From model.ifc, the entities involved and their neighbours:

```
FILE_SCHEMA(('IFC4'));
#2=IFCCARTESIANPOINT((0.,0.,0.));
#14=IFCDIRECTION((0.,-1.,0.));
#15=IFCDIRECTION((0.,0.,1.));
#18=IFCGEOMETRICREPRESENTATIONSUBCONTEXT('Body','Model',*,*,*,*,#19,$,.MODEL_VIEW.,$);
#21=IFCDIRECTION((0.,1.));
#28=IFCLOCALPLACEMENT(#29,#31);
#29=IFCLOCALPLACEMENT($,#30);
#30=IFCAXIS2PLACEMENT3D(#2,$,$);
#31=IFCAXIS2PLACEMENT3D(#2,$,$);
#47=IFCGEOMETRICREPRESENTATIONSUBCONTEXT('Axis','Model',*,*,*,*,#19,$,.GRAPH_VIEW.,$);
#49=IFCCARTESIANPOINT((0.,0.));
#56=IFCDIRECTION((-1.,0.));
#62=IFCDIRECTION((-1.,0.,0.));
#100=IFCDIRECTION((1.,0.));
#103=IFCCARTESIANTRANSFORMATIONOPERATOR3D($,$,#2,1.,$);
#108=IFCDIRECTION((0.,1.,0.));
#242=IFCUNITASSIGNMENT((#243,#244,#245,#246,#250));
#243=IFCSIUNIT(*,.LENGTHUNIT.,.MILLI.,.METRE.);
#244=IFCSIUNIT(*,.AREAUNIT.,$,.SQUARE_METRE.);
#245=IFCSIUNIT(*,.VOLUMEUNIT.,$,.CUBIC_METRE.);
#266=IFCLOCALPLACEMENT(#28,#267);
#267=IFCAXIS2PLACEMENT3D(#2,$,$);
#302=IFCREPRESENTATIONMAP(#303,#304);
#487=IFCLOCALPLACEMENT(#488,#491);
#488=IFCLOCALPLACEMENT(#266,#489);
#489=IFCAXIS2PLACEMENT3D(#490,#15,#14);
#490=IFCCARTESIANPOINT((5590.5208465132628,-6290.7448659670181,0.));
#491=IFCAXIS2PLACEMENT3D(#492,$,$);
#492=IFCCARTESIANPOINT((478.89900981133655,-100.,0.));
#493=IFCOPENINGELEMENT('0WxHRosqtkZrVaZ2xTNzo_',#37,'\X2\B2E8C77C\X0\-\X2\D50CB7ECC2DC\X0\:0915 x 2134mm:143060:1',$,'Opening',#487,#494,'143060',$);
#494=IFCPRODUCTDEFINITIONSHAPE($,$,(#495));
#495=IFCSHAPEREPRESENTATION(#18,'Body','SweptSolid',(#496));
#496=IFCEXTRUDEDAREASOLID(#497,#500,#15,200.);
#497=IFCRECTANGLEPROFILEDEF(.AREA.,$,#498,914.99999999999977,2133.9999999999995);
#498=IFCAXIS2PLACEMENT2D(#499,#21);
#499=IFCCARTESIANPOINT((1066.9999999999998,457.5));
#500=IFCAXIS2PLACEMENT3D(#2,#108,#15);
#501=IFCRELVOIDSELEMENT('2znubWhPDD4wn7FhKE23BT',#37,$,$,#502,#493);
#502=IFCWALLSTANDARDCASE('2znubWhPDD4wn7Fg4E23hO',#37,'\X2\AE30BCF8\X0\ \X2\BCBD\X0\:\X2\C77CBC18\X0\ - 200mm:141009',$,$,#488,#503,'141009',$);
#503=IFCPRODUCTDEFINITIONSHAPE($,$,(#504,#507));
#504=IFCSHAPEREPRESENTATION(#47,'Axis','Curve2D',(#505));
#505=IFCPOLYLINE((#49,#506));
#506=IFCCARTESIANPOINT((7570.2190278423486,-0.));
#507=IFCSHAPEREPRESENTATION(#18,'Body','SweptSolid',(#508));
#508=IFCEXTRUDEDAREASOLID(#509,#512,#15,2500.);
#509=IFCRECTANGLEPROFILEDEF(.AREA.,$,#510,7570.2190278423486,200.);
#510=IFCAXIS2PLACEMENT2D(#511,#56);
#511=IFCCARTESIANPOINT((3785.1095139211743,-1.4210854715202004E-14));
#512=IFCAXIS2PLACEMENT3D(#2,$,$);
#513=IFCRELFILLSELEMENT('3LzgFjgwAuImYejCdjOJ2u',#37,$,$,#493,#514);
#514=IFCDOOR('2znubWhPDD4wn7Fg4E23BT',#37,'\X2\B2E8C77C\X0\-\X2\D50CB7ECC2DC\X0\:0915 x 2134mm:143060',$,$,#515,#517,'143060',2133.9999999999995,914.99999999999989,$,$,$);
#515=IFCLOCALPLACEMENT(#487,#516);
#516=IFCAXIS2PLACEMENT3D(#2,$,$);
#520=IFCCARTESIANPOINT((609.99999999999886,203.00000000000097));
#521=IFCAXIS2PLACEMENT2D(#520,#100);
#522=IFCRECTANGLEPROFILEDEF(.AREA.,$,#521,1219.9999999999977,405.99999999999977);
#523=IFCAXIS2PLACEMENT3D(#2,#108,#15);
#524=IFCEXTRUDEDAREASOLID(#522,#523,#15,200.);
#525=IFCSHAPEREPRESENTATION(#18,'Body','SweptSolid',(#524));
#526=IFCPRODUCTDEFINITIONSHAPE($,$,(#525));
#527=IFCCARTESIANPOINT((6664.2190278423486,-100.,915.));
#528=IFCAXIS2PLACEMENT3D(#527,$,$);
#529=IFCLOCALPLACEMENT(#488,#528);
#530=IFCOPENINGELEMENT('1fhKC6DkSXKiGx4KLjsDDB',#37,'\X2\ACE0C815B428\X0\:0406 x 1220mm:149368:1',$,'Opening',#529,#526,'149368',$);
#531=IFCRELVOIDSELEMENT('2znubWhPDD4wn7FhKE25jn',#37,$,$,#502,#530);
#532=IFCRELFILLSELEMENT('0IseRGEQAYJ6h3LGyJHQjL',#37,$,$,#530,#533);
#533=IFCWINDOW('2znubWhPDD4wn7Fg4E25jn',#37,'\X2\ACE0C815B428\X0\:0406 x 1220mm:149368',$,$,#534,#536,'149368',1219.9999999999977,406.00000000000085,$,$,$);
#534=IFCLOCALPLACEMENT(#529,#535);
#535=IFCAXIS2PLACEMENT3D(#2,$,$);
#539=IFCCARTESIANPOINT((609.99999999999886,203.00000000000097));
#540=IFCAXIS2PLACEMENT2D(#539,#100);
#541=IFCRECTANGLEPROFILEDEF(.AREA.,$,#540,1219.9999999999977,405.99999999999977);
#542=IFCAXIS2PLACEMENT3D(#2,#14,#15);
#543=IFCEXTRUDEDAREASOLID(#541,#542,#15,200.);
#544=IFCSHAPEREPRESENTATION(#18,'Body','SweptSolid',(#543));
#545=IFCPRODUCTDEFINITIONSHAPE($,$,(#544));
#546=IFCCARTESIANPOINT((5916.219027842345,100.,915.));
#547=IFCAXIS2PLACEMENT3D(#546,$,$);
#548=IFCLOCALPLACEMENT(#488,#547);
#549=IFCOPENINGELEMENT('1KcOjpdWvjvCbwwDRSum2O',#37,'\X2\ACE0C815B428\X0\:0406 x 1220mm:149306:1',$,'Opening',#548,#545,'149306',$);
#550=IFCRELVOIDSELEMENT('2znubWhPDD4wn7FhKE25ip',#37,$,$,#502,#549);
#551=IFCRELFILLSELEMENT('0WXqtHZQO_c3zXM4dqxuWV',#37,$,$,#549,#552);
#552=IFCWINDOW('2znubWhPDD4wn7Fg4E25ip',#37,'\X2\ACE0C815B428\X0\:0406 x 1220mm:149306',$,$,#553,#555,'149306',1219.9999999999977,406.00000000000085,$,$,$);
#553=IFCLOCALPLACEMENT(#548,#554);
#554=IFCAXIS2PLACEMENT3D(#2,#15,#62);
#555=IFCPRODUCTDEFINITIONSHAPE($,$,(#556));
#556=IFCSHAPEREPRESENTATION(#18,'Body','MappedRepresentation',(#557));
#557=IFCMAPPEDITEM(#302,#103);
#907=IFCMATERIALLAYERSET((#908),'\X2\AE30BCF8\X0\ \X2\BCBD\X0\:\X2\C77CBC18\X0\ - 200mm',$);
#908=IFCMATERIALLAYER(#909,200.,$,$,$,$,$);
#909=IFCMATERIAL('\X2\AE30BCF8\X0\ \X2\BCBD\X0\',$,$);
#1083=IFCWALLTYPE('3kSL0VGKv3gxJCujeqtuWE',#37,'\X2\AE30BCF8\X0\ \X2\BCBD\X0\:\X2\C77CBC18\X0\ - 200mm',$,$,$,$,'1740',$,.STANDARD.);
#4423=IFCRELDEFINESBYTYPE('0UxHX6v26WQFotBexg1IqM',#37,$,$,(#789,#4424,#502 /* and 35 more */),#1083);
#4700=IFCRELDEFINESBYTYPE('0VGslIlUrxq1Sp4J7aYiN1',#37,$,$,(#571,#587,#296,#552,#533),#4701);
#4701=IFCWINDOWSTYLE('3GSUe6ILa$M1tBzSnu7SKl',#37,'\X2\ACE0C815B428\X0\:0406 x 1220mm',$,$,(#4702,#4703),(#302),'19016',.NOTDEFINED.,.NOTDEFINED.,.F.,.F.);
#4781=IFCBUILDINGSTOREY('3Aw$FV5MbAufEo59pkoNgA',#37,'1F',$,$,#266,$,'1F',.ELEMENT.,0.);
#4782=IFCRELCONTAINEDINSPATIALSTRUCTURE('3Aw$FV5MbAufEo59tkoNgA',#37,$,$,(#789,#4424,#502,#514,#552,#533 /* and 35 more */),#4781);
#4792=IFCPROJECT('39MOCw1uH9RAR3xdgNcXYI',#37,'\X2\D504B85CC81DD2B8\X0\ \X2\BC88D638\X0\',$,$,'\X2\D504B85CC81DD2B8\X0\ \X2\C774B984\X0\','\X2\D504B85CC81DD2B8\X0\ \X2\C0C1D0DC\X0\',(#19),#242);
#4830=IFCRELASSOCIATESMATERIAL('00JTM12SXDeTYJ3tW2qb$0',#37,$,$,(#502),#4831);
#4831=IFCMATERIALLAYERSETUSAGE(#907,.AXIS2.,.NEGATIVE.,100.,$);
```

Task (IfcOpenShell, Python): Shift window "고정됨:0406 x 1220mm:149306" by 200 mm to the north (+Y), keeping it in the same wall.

```python
import ifcopenshell
import ifcopenshell.api.geometry
import ifcopenshell.util.placement
import ifcopenshell.util.unit

model = ifcopenshell.open("model.ifc")
unit_scale = ifcopenshell.util.unit.calculate_unit_scale(model)

window = model.by_guid("2znubWhPDD4wn7Fg4E25ip")
opening = window.FillsVoids[0].RelatingOpeningElement
wall = opening.VoidsElements[0].RelatingBuildingElement

wall_matrix = ifcopenshell.util.placement.get_local_placement(wall.ObjectPlacement)
shift = wall_matrix[:3, 0] * -0.2 / unit_scale
before = ifcopenshell.util.placement.get_local_placement(window.ObjectPlacement)[:3, 3].copy()

# The window is placed relative to its opening, so it follows when the opening moves.
matrix = ifcopenshell.util.placement.get_local_placement(opening.ObjectPlacement)
matrix[:3, 3] += shift
ifcopenshell.api.geometry.edit_object_placement(
    model, product=opening, matrix=matrix, is_si=False, should_transform_children=True
)

after = ifcopenshell.util.placement.get_local_placement(window.ObjectPlacement)[:3, 3]
print("window moved by", (after - before).round(3) + 0.0)

model.write("model_updated.ifc")
```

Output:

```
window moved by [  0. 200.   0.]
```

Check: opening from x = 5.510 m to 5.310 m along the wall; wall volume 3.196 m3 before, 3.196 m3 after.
